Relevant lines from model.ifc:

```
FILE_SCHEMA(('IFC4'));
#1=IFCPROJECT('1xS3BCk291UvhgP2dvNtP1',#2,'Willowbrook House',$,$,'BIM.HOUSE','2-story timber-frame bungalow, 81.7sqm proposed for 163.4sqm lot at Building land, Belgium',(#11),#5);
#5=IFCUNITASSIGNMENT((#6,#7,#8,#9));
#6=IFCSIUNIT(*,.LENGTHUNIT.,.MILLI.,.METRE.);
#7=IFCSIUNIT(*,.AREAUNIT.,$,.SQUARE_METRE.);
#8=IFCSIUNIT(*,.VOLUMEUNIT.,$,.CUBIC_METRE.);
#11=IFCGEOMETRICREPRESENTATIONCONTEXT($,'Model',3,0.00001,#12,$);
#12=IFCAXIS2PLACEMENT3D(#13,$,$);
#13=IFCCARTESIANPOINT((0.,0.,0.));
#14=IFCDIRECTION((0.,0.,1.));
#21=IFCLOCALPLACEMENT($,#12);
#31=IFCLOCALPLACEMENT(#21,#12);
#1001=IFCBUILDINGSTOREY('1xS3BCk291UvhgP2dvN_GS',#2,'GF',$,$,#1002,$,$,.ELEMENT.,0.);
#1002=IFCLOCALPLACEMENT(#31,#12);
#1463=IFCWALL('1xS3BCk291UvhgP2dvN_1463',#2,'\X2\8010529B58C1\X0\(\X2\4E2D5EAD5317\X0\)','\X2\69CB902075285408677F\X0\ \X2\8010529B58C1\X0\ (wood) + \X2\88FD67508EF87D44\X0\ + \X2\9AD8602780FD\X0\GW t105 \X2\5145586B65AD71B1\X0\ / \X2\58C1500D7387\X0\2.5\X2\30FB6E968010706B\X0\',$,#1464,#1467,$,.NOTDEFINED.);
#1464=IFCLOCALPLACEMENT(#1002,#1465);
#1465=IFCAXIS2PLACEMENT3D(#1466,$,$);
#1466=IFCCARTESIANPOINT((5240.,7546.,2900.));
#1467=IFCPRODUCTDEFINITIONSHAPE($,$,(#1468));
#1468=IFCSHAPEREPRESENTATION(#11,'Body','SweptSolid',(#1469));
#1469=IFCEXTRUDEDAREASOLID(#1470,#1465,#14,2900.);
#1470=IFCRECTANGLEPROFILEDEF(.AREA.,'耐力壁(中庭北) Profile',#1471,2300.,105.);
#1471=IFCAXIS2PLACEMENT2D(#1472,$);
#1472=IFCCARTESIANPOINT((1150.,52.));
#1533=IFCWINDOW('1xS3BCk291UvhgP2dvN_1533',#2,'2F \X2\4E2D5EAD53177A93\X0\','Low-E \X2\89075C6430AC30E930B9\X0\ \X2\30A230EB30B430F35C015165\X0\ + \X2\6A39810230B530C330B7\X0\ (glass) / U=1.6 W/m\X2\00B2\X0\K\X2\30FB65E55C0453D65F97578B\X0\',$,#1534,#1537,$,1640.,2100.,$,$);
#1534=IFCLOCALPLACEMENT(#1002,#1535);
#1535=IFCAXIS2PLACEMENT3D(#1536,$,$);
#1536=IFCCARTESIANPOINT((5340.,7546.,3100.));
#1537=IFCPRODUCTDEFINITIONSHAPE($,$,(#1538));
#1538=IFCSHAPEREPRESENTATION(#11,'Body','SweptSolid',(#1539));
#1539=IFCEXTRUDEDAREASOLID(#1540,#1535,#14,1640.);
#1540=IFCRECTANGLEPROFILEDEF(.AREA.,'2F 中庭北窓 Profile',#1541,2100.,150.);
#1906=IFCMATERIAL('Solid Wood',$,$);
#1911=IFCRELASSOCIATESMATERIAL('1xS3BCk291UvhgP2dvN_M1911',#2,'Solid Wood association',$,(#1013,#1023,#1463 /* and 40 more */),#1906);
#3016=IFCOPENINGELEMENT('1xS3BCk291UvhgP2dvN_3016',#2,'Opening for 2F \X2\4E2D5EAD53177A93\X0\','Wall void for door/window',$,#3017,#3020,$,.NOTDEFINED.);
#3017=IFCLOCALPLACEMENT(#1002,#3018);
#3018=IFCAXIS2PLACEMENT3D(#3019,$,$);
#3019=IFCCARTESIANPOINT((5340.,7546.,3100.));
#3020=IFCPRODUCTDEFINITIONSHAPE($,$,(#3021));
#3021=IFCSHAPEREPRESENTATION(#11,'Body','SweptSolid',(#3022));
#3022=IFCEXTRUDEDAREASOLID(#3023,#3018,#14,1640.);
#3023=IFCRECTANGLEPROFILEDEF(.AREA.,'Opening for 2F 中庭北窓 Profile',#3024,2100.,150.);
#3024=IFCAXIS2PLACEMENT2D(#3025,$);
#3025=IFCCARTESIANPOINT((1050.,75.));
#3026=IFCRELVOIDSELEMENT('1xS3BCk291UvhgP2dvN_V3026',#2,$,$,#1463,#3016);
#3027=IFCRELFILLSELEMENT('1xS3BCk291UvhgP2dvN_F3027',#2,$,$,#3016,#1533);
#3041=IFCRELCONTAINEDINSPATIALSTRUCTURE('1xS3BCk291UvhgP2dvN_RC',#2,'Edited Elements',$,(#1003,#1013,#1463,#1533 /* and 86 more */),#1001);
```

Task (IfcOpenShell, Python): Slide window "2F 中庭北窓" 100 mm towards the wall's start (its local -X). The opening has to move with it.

```python
import ifcopenshell
import ifcopenshell.api.geometry
import ifcopenshell.util.placement

model = ifcopenshell.open("model.ifc")

window = model.by_id(1533)
opening = window.FillsVoids[0].RelatingOpeningElement
wall = opening.VoidsElements[0].RelatingBuildingElement

wall_matrix = ifcopenshell.util.placement.get_local_placement(wall.ObjectPlacement)
shift = wall_matrix[:3, 0] * -100.0
before = ifcopenshell.util.placement.get_local_placement(window.ObjectPlacement)[:3, 3].copy()

# The window is not placed relative to its opening, so move both.
for product in (opening, window):
    matrix = ifcopenshell.util.placement.get_local_placement(product.ObjectPlacement)
    matrix[:3, 3] += shift
    ifcopenshell.api.geometry.edit_object_placement(model, product=product, matrix=matrix, is_si=False)

after = ifcopenshell.util.placement.get_local_placement(window.ObjectPlacement)[:3, 3]
print("window moved by", (after - before).round(3) + 0.0)

model.write("model_updated.ifc")
```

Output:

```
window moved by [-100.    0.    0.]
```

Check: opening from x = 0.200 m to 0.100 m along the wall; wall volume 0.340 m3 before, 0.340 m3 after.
